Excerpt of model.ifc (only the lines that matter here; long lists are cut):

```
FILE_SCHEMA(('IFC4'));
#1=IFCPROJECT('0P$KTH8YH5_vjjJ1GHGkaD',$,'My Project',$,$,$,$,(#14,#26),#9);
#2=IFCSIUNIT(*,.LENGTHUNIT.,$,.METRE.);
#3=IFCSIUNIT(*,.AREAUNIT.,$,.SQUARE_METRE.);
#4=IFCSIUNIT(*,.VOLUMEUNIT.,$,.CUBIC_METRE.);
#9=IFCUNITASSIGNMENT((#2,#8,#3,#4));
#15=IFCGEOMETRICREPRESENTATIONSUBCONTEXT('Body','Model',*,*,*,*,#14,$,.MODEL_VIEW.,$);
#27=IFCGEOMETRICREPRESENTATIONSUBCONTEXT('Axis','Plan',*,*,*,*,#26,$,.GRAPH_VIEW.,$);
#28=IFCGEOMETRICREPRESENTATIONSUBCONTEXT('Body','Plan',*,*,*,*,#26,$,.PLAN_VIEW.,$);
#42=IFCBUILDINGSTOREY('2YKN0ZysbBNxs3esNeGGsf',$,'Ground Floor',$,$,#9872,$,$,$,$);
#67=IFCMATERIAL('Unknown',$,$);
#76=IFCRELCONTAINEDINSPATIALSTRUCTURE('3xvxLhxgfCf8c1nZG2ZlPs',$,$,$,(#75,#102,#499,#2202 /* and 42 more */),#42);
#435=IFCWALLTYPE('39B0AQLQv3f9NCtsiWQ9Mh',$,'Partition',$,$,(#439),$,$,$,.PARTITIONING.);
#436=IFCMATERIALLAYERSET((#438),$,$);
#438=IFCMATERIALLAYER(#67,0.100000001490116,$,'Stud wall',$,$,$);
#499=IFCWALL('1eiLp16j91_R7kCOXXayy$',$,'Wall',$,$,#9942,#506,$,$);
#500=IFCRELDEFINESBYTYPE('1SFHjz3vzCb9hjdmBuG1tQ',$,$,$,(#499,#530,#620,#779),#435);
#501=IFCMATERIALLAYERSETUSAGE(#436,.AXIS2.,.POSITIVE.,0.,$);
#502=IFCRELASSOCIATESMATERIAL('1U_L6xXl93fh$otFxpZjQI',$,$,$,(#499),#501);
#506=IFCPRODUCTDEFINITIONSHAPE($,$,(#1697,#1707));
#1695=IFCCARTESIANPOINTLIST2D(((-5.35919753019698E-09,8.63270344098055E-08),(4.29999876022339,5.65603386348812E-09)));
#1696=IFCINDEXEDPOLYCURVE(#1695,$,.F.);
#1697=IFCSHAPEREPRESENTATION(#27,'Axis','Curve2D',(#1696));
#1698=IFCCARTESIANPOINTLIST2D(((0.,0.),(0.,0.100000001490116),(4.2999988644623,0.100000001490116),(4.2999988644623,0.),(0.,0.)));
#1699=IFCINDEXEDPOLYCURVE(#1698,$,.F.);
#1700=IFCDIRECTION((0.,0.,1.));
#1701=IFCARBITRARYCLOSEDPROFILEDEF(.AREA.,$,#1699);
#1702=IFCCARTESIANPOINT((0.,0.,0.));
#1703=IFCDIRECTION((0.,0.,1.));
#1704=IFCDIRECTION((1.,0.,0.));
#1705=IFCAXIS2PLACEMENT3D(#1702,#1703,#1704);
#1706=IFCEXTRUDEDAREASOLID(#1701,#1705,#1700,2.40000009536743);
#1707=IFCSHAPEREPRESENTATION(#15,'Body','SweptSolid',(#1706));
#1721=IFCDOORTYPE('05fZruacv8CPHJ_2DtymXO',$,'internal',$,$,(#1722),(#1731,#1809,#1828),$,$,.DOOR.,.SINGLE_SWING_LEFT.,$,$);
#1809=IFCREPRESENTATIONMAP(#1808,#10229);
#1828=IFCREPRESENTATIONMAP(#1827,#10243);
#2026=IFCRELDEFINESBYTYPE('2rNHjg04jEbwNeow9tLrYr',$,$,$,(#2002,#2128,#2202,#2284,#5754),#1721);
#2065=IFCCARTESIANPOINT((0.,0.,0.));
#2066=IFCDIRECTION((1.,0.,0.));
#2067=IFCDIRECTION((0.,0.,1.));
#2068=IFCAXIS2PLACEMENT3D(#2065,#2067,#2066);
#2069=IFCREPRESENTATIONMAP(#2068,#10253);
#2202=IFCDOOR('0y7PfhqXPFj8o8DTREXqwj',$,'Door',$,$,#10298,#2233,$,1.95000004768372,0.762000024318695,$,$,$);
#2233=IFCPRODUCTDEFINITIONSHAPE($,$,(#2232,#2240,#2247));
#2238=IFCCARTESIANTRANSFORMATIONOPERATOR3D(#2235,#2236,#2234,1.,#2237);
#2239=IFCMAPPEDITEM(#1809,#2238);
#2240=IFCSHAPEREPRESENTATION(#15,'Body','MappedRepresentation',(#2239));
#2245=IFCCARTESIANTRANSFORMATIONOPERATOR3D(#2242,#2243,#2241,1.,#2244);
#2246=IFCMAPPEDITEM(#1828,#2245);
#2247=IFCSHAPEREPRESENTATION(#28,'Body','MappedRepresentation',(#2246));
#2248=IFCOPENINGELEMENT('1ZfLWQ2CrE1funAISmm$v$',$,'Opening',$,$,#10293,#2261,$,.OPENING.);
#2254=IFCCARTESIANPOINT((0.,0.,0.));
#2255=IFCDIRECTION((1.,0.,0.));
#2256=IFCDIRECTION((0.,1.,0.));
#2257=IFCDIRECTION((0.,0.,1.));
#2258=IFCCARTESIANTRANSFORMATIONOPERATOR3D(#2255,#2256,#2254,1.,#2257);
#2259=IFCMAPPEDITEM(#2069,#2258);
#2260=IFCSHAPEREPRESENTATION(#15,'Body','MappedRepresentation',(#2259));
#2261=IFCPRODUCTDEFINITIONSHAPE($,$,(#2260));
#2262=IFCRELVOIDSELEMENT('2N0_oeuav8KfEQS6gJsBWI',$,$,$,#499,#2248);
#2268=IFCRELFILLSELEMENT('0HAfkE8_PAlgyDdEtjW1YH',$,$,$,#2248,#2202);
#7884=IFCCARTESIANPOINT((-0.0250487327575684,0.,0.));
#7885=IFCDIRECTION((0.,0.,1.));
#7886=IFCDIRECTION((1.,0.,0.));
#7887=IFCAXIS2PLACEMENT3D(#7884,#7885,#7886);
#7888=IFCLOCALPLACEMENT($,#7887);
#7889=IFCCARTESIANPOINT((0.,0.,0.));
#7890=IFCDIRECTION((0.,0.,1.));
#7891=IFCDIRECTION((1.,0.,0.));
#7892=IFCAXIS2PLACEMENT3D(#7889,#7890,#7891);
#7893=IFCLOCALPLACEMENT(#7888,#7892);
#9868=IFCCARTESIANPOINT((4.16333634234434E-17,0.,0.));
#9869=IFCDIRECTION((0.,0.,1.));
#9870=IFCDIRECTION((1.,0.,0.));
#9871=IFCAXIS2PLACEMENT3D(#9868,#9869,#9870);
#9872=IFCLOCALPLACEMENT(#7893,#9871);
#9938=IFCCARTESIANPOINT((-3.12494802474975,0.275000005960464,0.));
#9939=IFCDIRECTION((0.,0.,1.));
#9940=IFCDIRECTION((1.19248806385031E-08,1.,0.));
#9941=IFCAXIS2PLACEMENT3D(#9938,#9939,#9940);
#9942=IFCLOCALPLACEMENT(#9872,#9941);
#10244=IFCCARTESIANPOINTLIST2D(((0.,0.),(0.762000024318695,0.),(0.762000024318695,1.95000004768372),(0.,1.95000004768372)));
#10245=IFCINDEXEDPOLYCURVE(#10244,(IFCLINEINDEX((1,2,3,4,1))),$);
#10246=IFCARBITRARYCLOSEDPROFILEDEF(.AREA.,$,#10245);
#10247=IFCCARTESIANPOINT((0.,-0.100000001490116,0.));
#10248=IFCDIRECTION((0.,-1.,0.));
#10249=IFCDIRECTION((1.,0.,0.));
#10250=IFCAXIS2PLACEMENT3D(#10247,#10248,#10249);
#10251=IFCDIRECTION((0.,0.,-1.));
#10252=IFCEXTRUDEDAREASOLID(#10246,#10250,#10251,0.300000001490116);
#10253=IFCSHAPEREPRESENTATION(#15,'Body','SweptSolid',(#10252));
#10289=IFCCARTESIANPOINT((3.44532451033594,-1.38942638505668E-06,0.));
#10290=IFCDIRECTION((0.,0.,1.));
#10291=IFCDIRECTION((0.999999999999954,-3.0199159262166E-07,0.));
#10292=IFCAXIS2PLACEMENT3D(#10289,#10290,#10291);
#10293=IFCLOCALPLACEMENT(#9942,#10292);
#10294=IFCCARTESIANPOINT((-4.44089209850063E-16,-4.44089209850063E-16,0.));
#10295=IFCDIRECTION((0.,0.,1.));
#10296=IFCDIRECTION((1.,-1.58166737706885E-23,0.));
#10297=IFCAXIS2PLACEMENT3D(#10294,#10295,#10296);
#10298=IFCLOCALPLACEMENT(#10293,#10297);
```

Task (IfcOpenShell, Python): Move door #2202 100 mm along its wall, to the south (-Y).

```python
import ifcopenshell
import ifcopenshell.api.geometry
import ifcopenshell.util.placement
import ifcopenshell.util.unit

model = ifcopenshell.open("model.ifc")
unit_scale = ifcopenshell.util.unit.calculate_unit_scale(model)

door = model.by_guid("0y7PfhqXPFj8o8DTREXqwj")
opening = door.FillsVoids[0].RelatingOpeningElement
wall = opening.VoidsElements[0].RelatingBuildingElement

wall_matrix = ifcopenshell.util.placement.get_local_placement(wall.ObjectPlacement)
shift = wall_matrix[:3, 0] * -0.1 / unit_scale
before = ifcopenshell.util.placement.get_local_placement(door.ObjectPlacement)[:3, 3].copy()

# The door is placed relative to its opening, so it follows when the opening moves.
matrix = ifcopenshell.util.placement.get_local_placement(opening.ObjectPlacement)
matrix[:3, 3] += shift
ifcopenshell.api.geometry.edit_object_placement(
    model, product=opening, matrix=matrix, is_si=False, should_transform_children=True
)

after = ifcopenshell.util.placement.get_local_placement(door.ObjectPlacement)[:3, 3]
print("door moved by", (after - before).round(3) + 0.0)

model.write("model_rev.ifc")
```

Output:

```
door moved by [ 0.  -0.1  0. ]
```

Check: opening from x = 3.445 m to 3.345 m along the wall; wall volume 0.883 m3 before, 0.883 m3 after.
